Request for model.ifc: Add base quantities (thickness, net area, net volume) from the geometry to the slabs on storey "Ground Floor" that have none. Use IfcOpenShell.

First a look at what the model holds.

```python
import ifcopenshell
import ifcopenshell.util.element
import ifcopenshell.util.unit

model = ifcopenshell.open("model.ifc")
print(model.schema)
for unit_type in ("LENGTHUNIT", "AREAUNIT", "VOLUMEUNIT"):
    print(unit_type, ifcopenshell.util.unit.calculate_unit_scale(model, unit_type))
storey = next(s for s in model.by_type("IfcBuildingStorey") if s.Name == "Ground Floor")
slabs = [e for e in ifcopenshell.util.element.get_decomposition(storey) if e.is_a("IfcSlab")]
for e in sorted(slabs, key=lambda e: e.id()):
    print(e.id(), e.is_a(), e.Name, list(ifcopenshell.util.element.get_psets(e, qtos_only=True)), sep=" | ")
```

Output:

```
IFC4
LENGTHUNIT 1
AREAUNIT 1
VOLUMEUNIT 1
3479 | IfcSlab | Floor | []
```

```python
import ifcopenshell
import ifcopenshell.api.pset
import ifcopenshell.geom
import ifcopenshell.util.element
import ifcopenshell.util.shape
import ifcopenshell.util.unit

model = ifcopenshell.open("model.ifc")
unit_scale = ifcopenshell.util.unit.calculate_unit_scale(model)
area_scale = ifcopenshell.util.unit.calculate_unit_scale(model, "AREAUNIT")
volume_scale = ifcopenshell.util.unit.calculate_unit_scale(model, "VOLUMEUNIT")
settings = ifcopenshell.geom.settings()

storey = next(s for s in model.by_type("IfcBuildingStorey") if s.Name == "Ground Floor")
slabs = [e for e in ifcopenshell.util.element.get_decomposition(storey) if e.is_a("IfcSlab")]

for e in sorted(slabs, key=lambda e: e.id()):
    if ifcopenshell.util.element.get_psets(e, qtos_only=True, should_inherit=False):
        continue
    # Geometry comes back in metres, in the element's own axes.
    shape = ifcopenshell.geom.create_shape(settings, e)
    values = {
        "Width": ifcopenshell.util.shape.get_z(shape.geometry) / unit_scale,
        "NetArea": ifcopenshell.util.shape.get_footprint_area(shape.geometry) / area_scale,
        "NetVolume": ifcopenshell.util.shape.get_volume(shape.geometry) / volume_scale,
    }
    qto = ifcopenshell.api.pset.add_qto(model, product=e, name="Qto_SlabBaseQuantities")
    ifcopenshell.api.pset.edit_qto(model, qto=qto, properties=values)
    print(e.id(), {k: round(v, 3) for k, v in values.items()})

model.write("model_edited.ifc")
```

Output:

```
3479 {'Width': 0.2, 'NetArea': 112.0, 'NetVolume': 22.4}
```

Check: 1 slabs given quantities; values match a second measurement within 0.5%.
